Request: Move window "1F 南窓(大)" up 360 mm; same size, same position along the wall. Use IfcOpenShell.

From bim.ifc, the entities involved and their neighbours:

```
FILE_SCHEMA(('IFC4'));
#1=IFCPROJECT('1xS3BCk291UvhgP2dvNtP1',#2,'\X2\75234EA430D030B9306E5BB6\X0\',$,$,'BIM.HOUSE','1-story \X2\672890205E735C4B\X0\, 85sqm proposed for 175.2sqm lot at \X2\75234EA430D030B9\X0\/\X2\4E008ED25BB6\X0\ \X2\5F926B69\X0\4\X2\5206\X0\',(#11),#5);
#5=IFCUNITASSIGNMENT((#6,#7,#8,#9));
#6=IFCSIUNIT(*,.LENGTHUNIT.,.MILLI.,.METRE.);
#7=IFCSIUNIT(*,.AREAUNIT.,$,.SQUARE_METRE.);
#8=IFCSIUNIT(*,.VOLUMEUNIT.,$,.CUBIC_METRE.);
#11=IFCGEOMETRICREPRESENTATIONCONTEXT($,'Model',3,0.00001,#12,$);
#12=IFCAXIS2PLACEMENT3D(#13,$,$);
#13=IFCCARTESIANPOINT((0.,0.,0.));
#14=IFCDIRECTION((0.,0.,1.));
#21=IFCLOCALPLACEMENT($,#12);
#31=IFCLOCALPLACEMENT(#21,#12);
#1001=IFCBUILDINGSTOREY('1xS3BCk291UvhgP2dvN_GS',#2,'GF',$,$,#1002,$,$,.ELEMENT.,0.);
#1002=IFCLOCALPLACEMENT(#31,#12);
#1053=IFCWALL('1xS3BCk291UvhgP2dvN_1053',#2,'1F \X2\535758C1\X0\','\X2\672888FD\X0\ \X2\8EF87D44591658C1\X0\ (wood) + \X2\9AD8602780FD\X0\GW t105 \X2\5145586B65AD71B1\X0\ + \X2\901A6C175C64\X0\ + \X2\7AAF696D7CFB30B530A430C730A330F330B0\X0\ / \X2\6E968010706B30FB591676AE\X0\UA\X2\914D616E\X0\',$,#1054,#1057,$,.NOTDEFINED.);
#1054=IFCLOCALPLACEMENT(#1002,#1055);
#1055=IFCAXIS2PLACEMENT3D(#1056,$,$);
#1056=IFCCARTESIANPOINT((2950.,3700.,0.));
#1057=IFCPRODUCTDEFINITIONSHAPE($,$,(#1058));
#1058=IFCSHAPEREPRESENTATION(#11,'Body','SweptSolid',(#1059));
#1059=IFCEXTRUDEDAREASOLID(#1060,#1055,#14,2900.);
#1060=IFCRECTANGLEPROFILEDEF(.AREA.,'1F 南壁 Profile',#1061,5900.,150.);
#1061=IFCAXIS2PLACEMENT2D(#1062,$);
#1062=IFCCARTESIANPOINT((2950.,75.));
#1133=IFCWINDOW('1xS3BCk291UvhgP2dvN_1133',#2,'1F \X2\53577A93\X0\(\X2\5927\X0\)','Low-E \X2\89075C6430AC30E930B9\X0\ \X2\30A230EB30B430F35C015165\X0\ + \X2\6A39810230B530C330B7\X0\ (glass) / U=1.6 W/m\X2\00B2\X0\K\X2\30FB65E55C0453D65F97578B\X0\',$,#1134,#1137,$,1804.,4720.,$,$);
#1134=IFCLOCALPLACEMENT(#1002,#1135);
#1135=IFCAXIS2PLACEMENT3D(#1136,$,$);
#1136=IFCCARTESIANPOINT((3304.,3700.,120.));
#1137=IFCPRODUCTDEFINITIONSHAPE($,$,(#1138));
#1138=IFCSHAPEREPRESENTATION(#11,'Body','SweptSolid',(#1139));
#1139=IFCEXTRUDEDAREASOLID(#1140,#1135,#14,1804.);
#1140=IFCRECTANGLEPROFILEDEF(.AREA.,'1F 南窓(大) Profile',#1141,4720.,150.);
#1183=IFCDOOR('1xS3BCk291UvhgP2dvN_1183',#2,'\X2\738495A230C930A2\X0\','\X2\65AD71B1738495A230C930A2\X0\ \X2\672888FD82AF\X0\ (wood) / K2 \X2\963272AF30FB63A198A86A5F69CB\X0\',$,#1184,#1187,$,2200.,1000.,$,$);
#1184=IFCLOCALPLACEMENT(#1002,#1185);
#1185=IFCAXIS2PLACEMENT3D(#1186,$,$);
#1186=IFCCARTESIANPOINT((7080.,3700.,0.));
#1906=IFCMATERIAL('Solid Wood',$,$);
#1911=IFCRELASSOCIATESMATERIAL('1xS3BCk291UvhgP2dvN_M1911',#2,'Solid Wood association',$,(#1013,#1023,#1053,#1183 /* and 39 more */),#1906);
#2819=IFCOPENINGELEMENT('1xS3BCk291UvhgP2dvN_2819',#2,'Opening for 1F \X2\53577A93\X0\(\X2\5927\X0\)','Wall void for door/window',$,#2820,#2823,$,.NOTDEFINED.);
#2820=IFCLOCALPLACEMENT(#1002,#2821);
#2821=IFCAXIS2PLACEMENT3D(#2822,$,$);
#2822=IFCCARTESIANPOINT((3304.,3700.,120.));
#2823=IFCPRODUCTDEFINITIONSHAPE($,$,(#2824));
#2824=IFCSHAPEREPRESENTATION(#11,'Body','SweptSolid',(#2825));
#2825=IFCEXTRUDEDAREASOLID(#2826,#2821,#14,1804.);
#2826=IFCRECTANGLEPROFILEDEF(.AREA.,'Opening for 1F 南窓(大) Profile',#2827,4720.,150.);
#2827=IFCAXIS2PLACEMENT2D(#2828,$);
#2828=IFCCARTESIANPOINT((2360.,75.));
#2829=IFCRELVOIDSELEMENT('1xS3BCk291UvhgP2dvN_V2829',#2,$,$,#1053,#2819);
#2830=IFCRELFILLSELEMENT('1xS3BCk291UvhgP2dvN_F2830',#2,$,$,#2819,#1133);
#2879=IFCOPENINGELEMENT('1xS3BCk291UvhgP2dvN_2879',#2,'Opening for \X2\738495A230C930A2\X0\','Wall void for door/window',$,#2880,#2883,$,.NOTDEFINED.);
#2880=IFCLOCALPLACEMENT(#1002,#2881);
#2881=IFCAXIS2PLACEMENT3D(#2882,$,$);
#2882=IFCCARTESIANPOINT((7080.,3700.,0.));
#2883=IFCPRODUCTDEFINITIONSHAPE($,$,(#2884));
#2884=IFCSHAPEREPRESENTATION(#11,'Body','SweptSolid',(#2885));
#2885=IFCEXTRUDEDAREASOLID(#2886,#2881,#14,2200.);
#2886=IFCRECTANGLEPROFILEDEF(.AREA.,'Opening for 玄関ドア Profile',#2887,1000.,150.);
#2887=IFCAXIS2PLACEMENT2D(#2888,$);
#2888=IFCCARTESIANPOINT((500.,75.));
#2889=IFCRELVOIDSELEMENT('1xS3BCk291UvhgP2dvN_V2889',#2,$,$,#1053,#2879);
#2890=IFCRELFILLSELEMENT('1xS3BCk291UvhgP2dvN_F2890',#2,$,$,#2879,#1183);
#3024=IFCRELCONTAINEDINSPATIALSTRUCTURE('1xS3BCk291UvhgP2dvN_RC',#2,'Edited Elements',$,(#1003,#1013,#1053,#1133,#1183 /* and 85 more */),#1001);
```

```python
import numpy as np
import ifcopenshell
import ifcopenshell.api.geometry
import ifcopenshell.util.placement
import ifcopenshell.util.unit

model = ifcopenshell.open("bim.ifc")
unit_scale = ifcopenshell.util.unit.calculate_unit_scale(model)

window = model.by_id(1133)
opening = window.FillsVoids[0].RelatingOpeningElement
dz = 0.36 / unit_scale

shift = np.array([0.0, 0.0, dz])
# The window is not placed relative to its opening, so move both.
for product in (opening, window):
    matrix = ifcopenshell.util.placement.get_local_placement(product.ObjectPlacement)
    matrix[:3, 3] += shift
    ifcopenshell.api.geometry.edit_object_placement(model, product=product, matrix=matrix, is_si=False)

print(f"moved by {dz * unit_scale:+.3f} m")

model.write("bim_edited.ifc")
```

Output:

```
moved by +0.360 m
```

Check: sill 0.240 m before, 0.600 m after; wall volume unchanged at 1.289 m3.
